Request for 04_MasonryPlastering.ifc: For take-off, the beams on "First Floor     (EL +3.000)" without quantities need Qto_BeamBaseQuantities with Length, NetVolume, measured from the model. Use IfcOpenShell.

First a look at what the model holds.

```python
import ifcopenshell
import ifcopenshell.util.element
import ifcopenshell.util.unit

model = ifcopenshell.open("04_MasonryPlastering.ifc")
print(model.schema)
for unit_type in ("LENGTHUNIT", "AREAUNIT", "VOLUMEUNIT"):
    print(unit_type, ifcopenshell.util.unit.calculate_unit_scale(model, unit_type))
storey = next(s for s in model.by_type("IfcBuildingStorey") if s.Name == "First Floor     (EL +3.000)")
beams = [e for e in ifcopenshell.util.element.get_decomposition(storey) if e.is_a("IfcBeam")]
for e in sorted(beams, key=lambda e: e.id()):
    print(e.id(), e.is_a(), e.Name, list(ifcopenshell.util.element.get_psets(e, qtos_only=True)), sep=" | ")
```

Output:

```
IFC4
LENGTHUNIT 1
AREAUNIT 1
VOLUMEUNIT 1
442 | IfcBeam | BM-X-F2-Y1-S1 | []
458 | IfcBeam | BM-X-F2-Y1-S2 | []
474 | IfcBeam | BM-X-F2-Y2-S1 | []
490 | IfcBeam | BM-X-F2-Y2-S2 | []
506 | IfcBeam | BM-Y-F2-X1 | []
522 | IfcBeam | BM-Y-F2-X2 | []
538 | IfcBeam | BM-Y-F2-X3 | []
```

```python
import ifcopenshell
import ifcopenshell.api.pset
import ifcopenshell.geom
import ifcopenshell.util.element
import ifcopenshell.util.shape
import ifcopenshell.util.unit

model = ifcopenshell.open("04_MasonryPlastering.ifc")
unit_scale = ifcopenshell.util.unit.calculate_unit_scale(model)
volume_scale = ifcopenshell.util.unit.calculate_unit_scale(model, "VOLUMEUNIT")
settings = ifcopenshell.geom.settings()

storey = next(s for s in model.by_type("IfcBuildingStorey") if s.Name == "First Floor     (EL +3.000)")
beams = [e for e in ifcopenshell.util.element.get_decomposition(storey) if e.is_a("IfcBeam")]

for e in sorted(beams, key=lambda e: e.id()):
    if ifcopenshell.util.element.get_psets(e, qtos_only=True, should_inherit=False):
        continue
    # Geometry comes back in metres, in the element's own axes.
    shape = ifcopenshell.geom.create_shape(settings, e)
    values = {
        "Length": ifcopenshell.util.shape.get_max_xyz(shape.geometry) / unit_scale,
        "NetVolume": ifcopenshell.util.shape.get_volume(shape.geometry) / volume_scale,
    }
    qto = ifcopenshell.api.pset.add_qto(model, product=e, name="Qto_BeamBaseQuantities")
    ifcopenshell.api.pset.edit_qto(model, qto=qto, properties=values)
    print(e.id(), {k: round(v, 3) for k, v in values.items()})

model.write("04_MasonryPlastering_v2.ifc")
```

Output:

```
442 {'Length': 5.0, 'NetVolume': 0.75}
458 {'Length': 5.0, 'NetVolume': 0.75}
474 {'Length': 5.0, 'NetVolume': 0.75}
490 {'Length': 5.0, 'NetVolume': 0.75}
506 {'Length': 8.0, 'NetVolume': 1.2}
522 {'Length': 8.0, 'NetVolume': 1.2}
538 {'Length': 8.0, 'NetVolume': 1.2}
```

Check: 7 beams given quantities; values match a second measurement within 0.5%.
